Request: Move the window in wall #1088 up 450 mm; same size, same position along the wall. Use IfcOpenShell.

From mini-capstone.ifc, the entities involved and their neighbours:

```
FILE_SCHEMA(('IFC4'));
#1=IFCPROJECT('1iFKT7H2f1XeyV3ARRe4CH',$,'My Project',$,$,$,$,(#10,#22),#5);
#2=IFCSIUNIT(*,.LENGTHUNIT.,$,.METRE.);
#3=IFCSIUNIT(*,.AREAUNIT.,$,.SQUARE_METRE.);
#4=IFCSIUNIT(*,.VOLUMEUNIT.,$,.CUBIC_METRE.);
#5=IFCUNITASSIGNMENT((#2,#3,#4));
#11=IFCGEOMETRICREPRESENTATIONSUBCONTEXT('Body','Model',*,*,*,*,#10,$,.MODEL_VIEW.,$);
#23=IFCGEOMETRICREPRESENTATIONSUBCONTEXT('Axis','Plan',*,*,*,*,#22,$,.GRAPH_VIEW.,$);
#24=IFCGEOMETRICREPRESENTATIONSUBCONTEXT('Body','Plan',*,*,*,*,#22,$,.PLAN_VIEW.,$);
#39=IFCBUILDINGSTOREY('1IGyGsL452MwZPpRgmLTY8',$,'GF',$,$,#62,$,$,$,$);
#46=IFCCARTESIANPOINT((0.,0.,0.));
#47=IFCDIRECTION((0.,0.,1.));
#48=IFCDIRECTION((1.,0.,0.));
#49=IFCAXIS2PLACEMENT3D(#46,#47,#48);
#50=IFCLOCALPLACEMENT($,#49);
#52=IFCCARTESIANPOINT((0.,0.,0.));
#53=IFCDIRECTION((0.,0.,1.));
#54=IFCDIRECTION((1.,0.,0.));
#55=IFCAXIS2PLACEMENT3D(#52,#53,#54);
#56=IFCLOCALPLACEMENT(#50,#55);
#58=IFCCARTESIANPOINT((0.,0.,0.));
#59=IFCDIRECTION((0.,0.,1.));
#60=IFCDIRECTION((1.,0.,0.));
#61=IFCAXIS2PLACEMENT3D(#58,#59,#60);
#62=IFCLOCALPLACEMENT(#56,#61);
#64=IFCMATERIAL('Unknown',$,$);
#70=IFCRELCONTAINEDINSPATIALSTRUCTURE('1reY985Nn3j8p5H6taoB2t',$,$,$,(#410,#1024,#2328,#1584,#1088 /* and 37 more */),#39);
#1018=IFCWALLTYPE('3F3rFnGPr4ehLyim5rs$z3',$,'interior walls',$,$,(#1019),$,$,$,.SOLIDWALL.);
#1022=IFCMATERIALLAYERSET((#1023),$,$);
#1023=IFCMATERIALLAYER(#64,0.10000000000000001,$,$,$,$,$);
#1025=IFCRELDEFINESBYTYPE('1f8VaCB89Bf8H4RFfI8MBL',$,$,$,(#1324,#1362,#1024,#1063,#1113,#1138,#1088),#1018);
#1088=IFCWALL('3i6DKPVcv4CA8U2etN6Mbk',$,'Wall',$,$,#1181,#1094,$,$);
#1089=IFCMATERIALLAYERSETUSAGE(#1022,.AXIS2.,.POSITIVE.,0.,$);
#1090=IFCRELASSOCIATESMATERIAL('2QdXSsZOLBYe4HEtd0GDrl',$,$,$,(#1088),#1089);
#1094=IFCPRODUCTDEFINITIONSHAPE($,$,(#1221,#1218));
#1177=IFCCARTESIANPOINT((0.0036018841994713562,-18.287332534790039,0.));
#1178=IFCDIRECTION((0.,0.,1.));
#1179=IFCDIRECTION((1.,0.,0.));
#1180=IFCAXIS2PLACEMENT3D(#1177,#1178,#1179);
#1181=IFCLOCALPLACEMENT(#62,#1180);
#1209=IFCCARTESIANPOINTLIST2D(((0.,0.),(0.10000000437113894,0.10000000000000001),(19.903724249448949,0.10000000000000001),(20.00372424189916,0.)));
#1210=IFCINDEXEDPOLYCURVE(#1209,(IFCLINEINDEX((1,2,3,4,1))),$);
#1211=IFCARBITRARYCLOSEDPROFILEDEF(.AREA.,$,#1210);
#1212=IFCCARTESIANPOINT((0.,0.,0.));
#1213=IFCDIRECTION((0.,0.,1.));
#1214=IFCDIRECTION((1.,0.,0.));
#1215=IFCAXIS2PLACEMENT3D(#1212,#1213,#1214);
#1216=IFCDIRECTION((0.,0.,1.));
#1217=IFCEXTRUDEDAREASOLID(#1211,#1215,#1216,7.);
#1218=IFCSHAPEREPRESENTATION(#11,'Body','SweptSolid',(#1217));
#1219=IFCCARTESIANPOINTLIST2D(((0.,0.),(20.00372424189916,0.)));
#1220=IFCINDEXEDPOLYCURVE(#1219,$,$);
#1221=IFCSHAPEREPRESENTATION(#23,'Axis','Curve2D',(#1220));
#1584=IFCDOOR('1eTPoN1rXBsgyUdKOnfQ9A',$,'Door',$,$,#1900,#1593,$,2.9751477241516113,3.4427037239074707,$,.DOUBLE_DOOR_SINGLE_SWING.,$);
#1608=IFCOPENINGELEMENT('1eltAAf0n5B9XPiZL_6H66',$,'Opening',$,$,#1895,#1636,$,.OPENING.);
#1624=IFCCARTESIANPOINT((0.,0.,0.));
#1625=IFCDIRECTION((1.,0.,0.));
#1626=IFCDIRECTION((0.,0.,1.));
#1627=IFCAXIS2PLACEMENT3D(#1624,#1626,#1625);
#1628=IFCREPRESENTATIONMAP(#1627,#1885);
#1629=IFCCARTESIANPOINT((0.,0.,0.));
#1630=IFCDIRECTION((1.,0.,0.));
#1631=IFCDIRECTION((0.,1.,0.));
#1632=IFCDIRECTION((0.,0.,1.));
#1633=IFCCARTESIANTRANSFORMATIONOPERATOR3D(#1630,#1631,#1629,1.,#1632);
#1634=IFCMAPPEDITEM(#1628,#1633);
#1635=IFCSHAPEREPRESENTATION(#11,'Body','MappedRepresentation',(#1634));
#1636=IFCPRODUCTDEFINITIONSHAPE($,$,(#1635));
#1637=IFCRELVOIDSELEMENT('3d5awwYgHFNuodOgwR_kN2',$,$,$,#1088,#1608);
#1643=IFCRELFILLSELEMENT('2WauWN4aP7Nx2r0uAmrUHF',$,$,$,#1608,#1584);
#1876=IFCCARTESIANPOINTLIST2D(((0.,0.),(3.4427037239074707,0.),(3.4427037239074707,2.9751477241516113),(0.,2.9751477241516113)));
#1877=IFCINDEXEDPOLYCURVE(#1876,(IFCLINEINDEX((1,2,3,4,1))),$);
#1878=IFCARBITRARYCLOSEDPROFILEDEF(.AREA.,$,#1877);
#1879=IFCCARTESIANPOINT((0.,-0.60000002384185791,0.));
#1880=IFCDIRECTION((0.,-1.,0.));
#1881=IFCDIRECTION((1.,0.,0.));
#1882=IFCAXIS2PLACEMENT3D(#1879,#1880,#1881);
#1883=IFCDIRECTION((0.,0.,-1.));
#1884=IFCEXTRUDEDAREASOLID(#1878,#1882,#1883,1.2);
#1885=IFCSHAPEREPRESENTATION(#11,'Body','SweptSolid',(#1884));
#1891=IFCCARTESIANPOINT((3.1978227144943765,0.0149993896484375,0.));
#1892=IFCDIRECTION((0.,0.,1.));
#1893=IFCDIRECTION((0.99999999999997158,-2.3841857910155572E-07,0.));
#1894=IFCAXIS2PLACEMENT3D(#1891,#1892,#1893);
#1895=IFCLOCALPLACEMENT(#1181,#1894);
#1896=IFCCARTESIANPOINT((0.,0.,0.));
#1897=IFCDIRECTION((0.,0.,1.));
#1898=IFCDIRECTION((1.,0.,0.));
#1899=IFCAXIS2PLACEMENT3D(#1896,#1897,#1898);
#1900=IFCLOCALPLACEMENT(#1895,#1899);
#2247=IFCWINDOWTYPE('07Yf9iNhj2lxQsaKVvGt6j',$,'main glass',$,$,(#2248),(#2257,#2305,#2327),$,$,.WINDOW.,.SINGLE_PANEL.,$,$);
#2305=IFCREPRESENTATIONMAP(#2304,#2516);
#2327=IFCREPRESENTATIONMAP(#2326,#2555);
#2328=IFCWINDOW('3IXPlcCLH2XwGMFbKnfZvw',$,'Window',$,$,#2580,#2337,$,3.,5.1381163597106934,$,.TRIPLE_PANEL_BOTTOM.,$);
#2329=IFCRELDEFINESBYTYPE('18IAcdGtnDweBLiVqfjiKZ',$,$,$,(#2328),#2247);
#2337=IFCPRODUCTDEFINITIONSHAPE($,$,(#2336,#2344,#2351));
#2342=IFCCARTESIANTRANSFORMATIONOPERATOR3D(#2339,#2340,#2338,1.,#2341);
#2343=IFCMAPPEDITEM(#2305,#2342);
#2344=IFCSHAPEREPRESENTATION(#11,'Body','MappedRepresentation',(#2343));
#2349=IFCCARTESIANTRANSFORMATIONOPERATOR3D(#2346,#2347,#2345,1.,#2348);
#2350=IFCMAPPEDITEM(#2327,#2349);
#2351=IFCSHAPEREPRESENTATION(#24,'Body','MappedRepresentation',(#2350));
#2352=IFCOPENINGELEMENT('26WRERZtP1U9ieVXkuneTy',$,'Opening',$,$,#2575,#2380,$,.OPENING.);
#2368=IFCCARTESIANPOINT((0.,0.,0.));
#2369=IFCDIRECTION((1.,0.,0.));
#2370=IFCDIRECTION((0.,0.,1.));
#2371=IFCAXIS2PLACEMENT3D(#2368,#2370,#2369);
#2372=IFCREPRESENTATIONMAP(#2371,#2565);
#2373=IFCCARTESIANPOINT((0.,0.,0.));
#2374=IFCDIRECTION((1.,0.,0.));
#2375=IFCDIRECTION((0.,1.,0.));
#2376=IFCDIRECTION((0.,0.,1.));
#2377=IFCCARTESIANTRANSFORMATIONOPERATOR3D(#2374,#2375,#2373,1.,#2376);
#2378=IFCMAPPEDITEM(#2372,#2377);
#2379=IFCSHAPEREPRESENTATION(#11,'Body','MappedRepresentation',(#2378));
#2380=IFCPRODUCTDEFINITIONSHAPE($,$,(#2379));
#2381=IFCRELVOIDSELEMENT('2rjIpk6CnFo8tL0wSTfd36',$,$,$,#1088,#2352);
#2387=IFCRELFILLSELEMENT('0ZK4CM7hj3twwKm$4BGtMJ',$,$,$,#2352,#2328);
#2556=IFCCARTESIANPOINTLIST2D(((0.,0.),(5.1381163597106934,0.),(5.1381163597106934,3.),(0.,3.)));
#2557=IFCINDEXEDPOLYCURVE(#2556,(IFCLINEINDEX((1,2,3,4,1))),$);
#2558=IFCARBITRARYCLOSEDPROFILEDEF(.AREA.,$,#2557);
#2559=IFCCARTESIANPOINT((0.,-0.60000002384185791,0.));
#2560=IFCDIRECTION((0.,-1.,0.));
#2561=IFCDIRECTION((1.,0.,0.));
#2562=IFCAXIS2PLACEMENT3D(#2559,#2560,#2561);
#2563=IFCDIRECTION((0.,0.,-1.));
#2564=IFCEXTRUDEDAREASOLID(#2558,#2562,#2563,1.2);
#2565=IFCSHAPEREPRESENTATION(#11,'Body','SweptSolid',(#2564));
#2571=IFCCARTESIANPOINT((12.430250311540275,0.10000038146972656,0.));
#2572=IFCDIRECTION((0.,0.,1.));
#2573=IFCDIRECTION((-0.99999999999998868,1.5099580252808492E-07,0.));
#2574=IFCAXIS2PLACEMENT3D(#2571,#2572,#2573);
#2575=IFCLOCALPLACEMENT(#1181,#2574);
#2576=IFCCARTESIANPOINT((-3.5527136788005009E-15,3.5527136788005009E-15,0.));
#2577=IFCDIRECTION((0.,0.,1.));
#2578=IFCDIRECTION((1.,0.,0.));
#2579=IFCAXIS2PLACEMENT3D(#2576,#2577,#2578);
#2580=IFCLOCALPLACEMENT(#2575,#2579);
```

```python
import numpy as np
import ifcopenshell
import ifcopenshell.api.geometry
import ifcopenshell.util.placement
import ifcopenshell.util.unit

model = ifcopenshell.open("mini-capstone.ifc")
unit_scale = ifcopenshell.util.unit.calculate_unit_scale(model)

window = model.by_guid("3IXPlcCLH2XwGMFbKnfZvw")
opening = window.FillsVoids[0].RelatingOpeningElement
dz = 0.45

shift = np.array([0.0, 0.0, dz])
# The window is placed relative to its opening, so it follows when the opening moves.
matrix = ifcopenshell.util.placement.get_local_placement(opening.ObjectPlacement)
matrix[:3, 3] += shift
ifcopenshell.api.geometry.edit_object_placement(
    model, product=opening, matrix=matrix, is_si=False, should_transform_children=True
)

print(f"moved by {dz * unit_scale:+.3f} m")

model.write("mini-capstone_edited.ifc")
```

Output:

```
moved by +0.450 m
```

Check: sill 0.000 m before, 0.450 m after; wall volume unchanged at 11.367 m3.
